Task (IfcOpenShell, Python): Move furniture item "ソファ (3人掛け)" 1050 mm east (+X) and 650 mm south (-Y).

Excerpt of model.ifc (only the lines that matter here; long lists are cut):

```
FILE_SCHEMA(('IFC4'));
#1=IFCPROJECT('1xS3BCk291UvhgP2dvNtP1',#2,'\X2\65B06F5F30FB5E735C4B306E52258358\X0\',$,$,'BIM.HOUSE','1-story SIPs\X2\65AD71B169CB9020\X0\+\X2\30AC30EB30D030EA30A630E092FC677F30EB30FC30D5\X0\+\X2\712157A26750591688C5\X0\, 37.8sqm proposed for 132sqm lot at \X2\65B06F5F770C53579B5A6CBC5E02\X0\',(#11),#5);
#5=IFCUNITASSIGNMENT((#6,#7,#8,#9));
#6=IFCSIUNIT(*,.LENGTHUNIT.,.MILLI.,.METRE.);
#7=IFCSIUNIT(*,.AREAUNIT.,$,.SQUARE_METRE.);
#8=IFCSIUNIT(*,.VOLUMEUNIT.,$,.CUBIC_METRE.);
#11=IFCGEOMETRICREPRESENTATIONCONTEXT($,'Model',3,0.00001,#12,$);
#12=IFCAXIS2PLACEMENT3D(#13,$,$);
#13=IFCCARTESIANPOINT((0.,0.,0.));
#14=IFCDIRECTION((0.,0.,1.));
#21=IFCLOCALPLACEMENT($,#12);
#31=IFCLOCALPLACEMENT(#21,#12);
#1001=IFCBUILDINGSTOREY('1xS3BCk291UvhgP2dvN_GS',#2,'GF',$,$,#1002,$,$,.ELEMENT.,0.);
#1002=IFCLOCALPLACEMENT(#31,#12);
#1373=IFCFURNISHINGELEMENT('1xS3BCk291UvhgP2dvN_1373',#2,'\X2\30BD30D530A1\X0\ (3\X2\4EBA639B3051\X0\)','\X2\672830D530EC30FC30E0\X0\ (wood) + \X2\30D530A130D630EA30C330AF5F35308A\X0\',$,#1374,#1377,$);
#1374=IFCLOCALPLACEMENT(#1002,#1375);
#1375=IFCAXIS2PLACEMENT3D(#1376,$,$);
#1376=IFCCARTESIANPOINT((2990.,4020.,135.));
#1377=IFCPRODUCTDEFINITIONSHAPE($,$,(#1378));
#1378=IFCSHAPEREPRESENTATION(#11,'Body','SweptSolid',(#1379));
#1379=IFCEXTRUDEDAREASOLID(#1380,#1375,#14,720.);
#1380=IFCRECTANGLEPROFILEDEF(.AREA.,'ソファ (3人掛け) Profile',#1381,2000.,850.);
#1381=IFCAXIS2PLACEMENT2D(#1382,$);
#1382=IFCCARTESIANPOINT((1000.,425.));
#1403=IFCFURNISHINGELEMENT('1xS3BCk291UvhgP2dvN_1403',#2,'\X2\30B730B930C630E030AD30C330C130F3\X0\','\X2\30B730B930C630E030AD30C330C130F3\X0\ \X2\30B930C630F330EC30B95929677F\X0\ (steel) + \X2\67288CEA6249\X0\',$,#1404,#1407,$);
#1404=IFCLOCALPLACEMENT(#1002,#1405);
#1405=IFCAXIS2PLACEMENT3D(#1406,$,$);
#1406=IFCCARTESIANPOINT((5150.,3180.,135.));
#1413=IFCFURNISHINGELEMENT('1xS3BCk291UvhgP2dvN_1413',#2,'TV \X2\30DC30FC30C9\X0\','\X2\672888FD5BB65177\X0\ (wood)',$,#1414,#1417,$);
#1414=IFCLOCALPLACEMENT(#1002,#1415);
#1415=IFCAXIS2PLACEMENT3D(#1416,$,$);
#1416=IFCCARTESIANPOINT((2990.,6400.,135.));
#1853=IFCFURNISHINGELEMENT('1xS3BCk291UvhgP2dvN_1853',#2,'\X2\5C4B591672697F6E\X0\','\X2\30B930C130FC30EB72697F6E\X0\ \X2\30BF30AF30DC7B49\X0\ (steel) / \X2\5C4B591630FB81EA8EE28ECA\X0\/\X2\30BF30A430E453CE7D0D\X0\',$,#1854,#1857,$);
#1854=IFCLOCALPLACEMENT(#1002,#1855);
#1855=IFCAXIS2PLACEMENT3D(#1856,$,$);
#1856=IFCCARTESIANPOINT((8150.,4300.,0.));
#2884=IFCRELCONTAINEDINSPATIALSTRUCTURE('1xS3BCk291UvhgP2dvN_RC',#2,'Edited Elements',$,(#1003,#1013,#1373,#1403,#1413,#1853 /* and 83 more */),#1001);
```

```python
import ifcopenshell
import ifcopenshell.api.geometry
import ifcopenshell.util.placement
import ifcopenshell.util.unit

model = ifcopenshell.open("model.ifc")
unit_scale = ifcopenshell.util.unit.calculate_unit_scale(model)

item = model.by_id(1373)
matrix = ifcopenshell.util.placement.get_local_placement(item.ObjectPlacement)
matrix[0, 3] += 1.05 / unit_scale
matrix[1, 3] -= 0.65 / unit_scale
ifcopenshell.api.geometry.edit_object_placement(model, product=item, matrix=matrix, is_si=False)

print(ifcopenshell.util.placement.get_local_placement(item.ObjectPlacement).round(3) + 0.0)

model.write("model_edited.ifc")
```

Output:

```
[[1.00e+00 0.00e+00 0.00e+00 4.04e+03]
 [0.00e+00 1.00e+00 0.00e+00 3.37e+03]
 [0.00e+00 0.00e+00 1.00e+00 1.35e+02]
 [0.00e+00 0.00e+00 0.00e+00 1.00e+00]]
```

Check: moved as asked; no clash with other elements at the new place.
